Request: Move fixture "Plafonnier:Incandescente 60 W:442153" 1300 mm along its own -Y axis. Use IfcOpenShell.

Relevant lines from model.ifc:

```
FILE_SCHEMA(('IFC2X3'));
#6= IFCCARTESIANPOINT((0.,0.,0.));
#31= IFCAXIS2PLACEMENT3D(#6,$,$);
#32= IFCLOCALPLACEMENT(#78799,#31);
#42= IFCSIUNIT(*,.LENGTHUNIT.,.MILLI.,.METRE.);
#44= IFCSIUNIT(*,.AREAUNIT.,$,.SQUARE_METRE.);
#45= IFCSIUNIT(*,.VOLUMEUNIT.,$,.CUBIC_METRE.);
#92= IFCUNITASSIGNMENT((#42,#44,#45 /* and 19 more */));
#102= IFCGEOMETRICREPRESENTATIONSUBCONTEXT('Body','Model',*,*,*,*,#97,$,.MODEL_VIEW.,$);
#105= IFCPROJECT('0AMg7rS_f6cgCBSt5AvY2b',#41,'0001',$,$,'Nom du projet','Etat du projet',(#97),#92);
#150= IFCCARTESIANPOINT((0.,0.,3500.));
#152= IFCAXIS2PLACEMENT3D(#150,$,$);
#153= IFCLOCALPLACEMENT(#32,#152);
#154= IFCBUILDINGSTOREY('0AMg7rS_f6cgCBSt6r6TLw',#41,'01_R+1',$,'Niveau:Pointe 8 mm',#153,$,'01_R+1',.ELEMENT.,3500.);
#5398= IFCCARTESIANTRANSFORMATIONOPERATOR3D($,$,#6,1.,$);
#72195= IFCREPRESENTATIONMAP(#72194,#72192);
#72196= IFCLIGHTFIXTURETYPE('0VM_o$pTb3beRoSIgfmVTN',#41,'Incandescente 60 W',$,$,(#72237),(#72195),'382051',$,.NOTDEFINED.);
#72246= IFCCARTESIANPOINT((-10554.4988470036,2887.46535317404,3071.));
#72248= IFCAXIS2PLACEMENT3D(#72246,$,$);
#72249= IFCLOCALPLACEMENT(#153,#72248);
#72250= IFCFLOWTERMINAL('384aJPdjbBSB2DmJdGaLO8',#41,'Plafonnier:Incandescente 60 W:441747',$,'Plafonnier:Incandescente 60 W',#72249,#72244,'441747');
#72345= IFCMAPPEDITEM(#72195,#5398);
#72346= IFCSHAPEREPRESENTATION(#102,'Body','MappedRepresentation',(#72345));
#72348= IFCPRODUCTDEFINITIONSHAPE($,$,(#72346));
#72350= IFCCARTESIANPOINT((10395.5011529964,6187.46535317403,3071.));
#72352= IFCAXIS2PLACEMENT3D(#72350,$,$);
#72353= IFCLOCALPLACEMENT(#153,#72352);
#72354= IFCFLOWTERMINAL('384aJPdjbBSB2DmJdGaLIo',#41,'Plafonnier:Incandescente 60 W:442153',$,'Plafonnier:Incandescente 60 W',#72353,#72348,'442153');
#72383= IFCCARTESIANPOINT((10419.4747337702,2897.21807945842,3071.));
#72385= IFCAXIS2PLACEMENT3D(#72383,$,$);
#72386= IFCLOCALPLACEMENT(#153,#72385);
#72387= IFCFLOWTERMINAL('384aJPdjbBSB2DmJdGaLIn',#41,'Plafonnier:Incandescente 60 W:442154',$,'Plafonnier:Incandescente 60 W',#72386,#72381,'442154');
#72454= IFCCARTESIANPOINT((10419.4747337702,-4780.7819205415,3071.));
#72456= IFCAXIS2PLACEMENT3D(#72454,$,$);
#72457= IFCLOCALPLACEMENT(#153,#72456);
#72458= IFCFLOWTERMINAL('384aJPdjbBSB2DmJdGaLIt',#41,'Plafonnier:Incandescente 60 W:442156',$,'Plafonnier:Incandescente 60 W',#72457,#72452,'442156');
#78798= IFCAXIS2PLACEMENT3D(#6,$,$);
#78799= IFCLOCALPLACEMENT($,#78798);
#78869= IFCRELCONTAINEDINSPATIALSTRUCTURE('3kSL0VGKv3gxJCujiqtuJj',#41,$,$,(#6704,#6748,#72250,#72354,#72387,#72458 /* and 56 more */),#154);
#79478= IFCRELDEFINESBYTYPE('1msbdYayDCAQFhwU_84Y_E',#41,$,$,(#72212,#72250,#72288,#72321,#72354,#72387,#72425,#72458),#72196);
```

```python
import ifcopenshell
import ifcopenshell.api.geometry
import ifcopenshell.util.placement
import ifcopenshell.util.unit

model = ifcopenshell.open("model.ifc")
unit_scale = ifcopenshell.util.unit.calculate_unit_scale(model)

item = model.by_guid("384aJPdjbBSB2DmJdGaLIo")
matrix = ifcopenshell.util.placement.get_local_placement(item.ObjectPlacement)
matrix[:3, 3] -= matrix[:3, 1] * 1.3 / unit_scale
ifcopenshell.api.geometry.edit_object_placement(model, product=item, matrix=matrix, is_si=False)

print(ifcopenshell.util.placement.get_local_placement(item.ObjectPlacement).round(3) + 0.0)

model.write("model_rev.ifc")
```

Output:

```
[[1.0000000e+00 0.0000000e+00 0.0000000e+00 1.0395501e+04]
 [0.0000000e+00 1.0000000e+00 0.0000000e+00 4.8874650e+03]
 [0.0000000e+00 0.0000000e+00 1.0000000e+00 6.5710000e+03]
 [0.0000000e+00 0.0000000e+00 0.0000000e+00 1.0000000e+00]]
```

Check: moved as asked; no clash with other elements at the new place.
